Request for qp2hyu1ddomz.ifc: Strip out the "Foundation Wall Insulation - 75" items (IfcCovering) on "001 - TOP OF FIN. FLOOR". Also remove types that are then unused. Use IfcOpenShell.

First a look at what the model holds.

```python
import ifcopenshell
import ifcopenshell.util.element

model = ifcopenshell.open("qp2hyu1ddomz.ifc")
print(model.schema)
storey = next(s for s in model.by_type("IfcBuildingStorey") if s.Name == "001 - TOP OF FIN. FLOOR")
coverings = [e for e in ifcopenshell.util.element.get_decomposition(storey) if e.is_a("IfcCovering")]
seen = {}
for e in coverings:
    element_type = ifcopenshell.util.element.get_type(e)
    name = element_type.Name if element_type not in (None, e) else None
    seen[name] = seen.get(name, 0) + 1
for name, count in sorted(seen.items(), key=str):
    print(count, "x", name)
```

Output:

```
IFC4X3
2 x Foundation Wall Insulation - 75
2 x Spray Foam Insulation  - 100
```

```python
import ifcopenshell
import ifcopenshell.api.root
import ifcopenshell.util.element

model = ifcopenshell.open("qp2hyu1ddomz.ifc")

storey = next(s for s in model.by_type("IfcBuildingStorey") if s.Name == "001 - TOP OF FIN. FLOOR")
coverings = [e for e in ifcopenshell.util.element.get_decomposition(storey) if e.is_a("IfcCovering")]
targets = [e for e in coverings if (t := ifcopenshell.util.element.get_type(e)) not in (None, e) and t.Name == "Foundation Wall Insulation - 75"]
types = {ifcopenshell.util.element.get_type(e) for e in targets} - {None, *targets}

for e in targets:
    ifcopenshell.api.root.remove_product(model, product=e)
print(len(targets), "removed")

unused = [t for t in types if not ifcopenshell.util.element.get_types(t)]
for t in unused:
    ifcopenshell.api.root.remove_product(model, product=t)
print(len(unused), "unused types removed")

model.write("qp2hyu1ddomz_edited.ifc")
```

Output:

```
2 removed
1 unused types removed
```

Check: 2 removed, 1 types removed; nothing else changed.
